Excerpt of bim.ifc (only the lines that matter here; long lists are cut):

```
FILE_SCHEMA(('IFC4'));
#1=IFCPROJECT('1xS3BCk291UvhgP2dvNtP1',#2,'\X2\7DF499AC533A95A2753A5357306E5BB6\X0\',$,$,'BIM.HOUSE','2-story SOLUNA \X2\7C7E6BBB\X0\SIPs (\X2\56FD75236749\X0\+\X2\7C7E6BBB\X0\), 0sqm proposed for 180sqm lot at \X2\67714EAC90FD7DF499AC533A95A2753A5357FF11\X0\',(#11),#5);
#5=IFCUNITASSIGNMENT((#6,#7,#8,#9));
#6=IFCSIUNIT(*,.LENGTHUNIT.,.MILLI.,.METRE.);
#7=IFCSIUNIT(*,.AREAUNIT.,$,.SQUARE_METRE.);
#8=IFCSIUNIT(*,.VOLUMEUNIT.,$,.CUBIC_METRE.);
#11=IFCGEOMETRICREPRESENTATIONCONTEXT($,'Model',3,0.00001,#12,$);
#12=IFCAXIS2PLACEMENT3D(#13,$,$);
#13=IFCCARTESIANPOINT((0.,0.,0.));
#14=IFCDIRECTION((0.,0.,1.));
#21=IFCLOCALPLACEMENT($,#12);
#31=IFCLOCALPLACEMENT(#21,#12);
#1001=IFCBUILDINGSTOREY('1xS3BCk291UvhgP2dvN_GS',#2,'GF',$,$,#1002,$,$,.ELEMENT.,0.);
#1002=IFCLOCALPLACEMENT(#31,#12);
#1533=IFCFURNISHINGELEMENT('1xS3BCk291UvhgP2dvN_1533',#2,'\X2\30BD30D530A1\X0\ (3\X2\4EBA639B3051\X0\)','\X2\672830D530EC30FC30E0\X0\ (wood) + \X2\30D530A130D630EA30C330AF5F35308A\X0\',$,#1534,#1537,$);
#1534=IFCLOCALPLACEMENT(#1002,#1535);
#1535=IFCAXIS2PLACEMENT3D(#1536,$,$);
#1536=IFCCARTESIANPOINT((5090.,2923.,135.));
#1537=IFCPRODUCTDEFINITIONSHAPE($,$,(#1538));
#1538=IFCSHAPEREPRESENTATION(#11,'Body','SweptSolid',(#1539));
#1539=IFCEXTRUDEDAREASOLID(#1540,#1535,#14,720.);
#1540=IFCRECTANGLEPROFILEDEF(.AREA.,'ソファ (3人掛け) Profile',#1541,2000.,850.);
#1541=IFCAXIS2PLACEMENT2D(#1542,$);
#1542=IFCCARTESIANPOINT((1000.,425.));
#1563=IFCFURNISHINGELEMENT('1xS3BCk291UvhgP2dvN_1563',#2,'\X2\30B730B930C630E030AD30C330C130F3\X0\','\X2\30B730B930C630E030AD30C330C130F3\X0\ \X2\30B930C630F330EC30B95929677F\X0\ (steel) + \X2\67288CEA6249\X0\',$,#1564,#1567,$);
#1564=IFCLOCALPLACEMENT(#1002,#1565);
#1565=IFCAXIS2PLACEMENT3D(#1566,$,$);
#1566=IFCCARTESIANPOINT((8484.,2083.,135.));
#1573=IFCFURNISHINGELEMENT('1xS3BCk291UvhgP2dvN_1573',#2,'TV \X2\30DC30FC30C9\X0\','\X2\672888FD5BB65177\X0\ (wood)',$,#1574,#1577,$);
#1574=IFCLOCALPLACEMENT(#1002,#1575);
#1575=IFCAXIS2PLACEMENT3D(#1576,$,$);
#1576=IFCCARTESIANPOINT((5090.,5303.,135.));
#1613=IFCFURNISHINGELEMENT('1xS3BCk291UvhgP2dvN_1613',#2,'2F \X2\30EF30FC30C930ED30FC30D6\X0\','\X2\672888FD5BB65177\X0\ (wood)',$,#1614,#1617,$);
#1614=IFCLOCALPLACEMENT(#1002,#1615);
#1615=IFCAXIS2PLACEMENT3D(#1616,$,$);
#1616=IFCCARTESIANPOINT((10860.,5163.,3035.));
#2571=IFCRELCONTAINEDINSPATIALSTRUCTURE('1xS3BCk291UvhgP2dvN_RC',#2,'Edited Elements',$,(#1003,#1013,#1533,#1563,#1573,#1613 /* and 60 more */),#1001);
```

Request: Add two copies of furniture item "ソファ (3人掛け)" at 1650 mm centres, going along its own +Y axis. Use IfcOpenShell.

```python
import ifcopenshell
import ifcopenshell.api.geometry
import ifcopenshell.api.root
import ifcopenshell.util.element
import ifcopenshell.util.placement

model = ifcopenshell.open("bim.ifc")


def reuse_history(source, copy):
    """copy_class also copies each property set's owner history, people and application; keep the originals."""
    for rel in copy.IsDefinedBy:
        if rel.is_a("IfcRelDefinesByProperties") and (history := rel.RelatingPropertyDefinition.OwnerHistory):
            rel.RelatingPropertyDefinition.OwnerHistory = source.OwnerHistory
            ifcopenshell.util.element.remove_deep2(model, history)


source = model.by_id(1533)
base = ifcopenshell.util.placement.get_local_placement(source.ObjectPlacement)
step = base[:3, 1] * 1650.0

for i in range(1, 3):
    copy = ifcopenshell.api.root.copy_class(model, product=source)
    copy.Representation = ifcopenshell.util.element.copy_deep(
        model, source.Representation, exclude=["IfcGeometricRepresentationContext", "IfcRepresentationMap"]
    )
    reuse_history(source, copy)
    matrix = base.copy()
    matrix[:3, 3] += i * step
    print("added at", matrix[:3, 3].round(3) + 0.0)
    ifcopenshell.api.geometry.edit_object_placement(model, product=copy, matrix=matrix, is_si=False)

model.write("bim-out.ifc")
```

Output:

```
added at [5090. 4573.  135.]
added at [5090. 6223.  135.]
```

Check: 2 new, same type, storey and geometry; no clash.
